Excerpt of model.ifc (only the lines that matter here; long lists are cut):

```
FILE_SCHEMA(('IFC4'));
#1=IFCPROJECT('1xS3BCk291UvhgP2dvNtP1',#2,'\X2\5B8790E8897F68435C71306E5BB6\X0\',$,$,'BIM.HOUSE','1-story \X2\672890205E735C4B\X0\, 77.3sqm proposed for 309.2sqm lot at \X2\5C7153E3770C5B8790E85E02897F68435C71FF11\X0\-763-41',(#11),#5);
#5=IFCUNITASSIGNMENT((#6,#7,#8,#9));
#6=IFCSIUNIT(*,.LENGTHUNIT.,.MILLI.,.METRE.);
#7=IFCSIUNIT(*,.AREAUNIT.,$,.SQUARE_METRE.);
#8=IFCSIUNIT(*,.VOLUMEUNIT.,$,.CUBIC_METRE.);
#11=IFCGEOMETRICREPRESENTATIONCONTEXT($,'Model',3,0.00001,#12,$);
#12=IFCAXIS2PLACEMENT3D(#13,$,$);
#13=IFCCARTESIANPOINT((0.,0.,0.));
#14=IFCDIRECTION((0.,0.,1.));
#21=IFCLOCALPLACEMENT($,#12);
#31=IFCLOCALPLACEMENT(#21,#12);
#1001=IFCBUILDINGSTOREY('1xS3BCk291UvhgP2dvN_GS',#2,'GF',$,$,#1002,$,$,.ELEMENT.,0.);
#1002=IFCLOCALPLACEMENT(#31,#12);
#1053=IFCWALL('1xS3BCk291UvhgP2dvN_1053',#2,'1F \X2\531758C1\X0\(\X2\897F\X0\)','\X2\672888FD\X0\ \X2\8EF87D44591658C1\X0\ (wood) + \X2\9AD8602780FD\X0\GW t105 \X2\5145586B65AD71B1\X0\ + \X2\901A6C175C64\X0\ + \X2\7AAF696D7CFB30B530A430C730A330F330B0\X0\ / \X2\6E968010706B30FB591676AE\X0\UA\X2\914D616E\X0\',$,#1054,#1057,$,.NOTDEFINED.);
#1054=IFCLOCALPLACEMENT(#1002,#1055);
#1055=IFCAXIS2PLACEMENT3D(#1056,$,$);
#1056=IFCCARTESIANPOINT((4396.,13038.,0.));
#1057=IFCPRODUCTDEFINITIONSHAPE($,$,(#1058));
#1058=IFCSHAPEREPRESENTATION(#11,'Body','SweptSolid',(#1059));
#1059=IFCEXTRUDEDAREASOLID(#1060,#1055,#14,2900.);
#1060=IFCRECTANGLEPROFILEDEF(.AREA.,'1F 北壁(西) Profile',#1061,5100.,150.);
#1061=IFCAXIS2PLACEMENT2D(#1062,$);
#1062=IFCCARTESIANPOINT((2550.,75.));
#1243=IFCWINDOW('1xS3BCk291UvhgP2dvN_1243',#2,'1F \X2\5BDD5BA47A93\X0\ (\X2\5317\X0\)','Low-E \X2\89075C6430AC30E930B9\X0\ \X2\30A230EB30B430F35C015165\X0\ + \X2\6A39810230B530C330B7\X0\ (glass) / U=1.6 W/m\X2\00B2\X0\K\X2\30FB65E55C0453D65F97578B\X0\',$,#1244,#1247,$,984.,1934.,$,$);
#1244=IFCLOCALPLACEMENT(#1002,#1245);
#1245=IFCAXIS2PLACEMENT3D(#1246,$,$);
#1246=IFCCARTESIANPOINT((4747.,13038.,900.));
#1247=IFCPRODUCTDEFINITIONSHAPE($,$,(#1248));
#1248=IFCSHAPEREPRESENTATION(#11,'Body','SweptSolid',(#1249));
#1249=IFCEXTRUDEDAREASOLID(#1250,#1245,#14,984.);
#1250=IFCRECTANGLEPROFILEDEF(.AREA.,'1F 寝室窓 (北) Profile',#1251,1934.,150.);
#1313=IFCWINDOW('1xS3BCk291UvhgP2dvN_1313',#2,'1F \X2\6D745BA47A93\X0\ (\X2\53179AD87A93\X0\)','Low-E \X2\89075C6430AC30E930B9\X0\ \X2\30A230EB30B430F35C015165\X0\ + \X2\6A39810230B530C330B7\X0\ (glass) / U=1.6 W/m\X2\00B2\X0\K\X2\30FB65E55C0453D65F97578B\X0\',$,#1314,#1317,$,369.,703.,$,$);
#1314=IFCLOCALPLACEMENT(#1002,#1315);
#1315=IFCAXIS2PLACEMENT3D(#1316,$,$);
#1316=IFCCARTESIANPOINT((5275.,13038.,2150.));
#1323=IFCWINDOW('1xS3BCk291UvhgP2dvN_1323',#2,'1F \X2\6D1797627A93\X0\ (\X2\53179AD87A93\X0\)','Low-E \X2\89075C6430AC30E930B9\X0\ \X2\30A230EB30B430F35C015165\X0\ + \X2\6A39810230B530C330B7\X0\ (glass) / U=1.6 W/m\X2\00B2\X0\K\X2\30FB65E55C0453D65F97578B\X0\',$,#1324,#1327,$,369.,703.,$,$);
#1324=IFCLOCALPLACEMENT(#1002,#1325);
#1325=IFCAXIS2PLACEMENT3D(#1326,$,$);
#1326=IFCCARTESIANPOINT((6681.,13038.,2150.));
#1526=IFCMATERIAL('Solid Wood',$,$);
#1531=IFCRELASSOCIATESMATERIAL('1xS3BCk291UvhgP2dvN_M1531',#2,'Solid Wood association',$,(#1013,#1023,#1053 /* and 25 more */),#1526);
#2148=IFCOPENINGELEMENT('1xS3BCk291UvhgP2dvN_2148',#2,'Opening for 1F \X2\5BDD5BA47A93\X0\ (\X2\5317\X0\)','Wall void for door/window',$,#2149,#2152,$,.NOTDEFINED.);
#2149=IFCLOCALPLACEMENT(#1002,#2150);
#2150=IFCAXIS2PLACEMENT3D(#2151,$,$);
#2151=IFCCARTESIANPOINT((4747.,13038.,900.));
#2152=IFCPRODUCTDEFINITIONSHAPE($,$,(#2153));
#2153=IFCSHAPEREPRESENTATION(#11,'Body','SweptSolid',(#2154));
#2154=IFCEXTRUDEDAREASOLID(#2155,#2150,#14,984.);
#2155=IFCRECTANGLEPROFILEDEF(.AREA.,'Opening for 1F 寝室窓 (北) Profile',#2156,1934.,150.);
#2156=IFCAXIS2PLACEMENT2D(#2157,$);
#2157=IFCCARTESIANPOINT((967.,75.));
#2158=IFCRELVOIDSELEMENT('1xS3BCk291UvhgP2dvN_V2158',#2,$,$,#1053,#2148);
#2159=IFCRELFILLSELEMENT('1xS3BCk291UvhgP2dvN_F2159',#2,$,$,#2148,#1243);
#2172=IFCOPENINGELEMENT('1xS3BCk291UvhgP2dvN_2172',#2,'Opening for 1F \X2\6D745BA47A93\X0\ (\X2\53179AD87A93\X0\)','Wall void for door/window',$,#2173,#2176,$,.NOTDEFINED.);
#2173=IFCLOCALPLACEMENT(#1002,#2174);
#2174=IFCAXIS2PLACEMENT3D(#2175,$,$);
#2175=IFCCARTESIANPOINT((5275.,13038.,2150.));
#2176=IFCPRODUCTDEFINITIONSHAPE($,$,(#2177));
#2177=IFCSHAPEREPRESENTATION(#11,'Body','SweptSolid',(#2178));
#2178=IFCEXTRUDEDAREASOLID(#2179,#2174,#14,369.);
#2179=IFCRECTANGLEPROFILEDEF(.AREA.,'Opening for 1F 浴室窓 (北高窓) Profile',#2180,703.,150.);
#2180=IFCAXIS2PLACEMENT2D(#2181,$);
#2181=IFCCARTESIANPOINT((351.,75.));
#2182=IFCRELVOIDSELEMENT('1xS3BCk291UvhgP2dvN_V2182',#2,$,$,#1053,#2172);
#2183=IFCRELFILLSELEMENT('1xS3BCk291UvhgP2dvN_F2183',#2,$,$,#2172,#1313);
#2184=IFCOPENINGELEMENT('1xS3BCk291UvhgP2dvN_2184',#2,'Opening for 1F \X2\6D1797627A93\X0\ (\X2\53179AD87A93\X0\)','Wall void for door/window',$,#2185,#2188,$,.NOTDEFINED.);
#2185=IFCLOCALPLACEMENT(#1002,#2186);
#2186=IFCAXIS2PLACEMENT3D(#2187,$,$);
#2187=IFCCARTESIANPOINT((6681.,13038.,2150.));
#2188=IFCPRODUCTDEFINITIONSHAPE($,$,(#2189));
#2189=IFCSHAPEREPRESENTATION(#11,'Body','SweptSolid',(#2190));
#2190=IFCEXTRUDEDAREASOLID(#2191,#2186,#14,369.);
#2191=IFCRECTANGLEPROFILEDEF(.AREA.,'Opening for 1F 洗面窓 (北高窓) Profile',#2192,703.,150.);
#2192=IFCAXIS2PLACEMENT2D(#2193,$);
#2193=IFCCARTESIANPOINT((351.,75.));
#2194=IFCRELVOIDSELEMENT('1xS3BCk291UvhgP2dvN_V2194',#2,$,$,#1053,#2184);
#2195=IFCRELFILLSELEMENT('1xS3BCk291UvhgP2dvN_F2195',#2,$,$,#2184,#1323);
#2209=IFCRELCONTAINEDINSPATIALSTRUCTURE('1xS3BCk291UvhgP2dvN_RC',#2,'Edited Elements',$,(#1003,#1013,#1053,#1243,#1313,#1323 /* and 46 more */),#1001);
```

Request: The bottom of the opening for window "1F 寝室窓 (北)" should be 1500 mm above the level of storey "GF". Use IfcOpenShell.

```python
import numpy as np
import ifcopenshell
import ifcopenshell.api.geometry
import ifcopenshell.geom
import ifcopenshell.util.element
import ifcopenshell.util.placement
import ifcopenshell.util.shape
import ifcopenshell.util.unit

model = ifcopenshell.open("model.ifc")
unit_scale = ifcopenshell.util.unit.calculate_unit_scale(model)

window = model.by_id(1243)
opening = window.FillsVoids[0].RelatingOpeningElement
storey = ifcopenshell.util.element.get_container(window, ifc_class="IfcBuildingStorey")
level = ifcopenshell.util.placement.get_local_placement(storey.ObjectPlacement)[2, 3]

# The opening's origin need not be at the sill, so measure its lowest point.
shape = ifcopenshell.geom.create_shape(ifcopenshell.geom.settings(), opening)
bottom = ifcopenshell.util.shape.get_shape_bottom_elevation(shape, shape.geometry) / unit_scale
dz = level + 1.5 / unit_scale - bottom

shift = np.array([0.0, 0.0, dz])
# The window is not placed relative to its opening, so move both.
for product in (opening, window):
    matrix = ifcopenshell.util.placement.get_local_placement(product.ObjectPlacement)
    matrix[:3, 3] += shift
    ifcopenshell.api.geometry.edit_object_placement(model, product=product, matrix=matrix, is_si=False)

print(f"moved by {dz * unit_scale:+.3f} m")

model.write("model_edited.ifc")
```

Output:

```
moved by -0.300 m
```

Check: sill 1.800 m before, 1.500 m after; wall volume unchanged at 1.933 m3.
